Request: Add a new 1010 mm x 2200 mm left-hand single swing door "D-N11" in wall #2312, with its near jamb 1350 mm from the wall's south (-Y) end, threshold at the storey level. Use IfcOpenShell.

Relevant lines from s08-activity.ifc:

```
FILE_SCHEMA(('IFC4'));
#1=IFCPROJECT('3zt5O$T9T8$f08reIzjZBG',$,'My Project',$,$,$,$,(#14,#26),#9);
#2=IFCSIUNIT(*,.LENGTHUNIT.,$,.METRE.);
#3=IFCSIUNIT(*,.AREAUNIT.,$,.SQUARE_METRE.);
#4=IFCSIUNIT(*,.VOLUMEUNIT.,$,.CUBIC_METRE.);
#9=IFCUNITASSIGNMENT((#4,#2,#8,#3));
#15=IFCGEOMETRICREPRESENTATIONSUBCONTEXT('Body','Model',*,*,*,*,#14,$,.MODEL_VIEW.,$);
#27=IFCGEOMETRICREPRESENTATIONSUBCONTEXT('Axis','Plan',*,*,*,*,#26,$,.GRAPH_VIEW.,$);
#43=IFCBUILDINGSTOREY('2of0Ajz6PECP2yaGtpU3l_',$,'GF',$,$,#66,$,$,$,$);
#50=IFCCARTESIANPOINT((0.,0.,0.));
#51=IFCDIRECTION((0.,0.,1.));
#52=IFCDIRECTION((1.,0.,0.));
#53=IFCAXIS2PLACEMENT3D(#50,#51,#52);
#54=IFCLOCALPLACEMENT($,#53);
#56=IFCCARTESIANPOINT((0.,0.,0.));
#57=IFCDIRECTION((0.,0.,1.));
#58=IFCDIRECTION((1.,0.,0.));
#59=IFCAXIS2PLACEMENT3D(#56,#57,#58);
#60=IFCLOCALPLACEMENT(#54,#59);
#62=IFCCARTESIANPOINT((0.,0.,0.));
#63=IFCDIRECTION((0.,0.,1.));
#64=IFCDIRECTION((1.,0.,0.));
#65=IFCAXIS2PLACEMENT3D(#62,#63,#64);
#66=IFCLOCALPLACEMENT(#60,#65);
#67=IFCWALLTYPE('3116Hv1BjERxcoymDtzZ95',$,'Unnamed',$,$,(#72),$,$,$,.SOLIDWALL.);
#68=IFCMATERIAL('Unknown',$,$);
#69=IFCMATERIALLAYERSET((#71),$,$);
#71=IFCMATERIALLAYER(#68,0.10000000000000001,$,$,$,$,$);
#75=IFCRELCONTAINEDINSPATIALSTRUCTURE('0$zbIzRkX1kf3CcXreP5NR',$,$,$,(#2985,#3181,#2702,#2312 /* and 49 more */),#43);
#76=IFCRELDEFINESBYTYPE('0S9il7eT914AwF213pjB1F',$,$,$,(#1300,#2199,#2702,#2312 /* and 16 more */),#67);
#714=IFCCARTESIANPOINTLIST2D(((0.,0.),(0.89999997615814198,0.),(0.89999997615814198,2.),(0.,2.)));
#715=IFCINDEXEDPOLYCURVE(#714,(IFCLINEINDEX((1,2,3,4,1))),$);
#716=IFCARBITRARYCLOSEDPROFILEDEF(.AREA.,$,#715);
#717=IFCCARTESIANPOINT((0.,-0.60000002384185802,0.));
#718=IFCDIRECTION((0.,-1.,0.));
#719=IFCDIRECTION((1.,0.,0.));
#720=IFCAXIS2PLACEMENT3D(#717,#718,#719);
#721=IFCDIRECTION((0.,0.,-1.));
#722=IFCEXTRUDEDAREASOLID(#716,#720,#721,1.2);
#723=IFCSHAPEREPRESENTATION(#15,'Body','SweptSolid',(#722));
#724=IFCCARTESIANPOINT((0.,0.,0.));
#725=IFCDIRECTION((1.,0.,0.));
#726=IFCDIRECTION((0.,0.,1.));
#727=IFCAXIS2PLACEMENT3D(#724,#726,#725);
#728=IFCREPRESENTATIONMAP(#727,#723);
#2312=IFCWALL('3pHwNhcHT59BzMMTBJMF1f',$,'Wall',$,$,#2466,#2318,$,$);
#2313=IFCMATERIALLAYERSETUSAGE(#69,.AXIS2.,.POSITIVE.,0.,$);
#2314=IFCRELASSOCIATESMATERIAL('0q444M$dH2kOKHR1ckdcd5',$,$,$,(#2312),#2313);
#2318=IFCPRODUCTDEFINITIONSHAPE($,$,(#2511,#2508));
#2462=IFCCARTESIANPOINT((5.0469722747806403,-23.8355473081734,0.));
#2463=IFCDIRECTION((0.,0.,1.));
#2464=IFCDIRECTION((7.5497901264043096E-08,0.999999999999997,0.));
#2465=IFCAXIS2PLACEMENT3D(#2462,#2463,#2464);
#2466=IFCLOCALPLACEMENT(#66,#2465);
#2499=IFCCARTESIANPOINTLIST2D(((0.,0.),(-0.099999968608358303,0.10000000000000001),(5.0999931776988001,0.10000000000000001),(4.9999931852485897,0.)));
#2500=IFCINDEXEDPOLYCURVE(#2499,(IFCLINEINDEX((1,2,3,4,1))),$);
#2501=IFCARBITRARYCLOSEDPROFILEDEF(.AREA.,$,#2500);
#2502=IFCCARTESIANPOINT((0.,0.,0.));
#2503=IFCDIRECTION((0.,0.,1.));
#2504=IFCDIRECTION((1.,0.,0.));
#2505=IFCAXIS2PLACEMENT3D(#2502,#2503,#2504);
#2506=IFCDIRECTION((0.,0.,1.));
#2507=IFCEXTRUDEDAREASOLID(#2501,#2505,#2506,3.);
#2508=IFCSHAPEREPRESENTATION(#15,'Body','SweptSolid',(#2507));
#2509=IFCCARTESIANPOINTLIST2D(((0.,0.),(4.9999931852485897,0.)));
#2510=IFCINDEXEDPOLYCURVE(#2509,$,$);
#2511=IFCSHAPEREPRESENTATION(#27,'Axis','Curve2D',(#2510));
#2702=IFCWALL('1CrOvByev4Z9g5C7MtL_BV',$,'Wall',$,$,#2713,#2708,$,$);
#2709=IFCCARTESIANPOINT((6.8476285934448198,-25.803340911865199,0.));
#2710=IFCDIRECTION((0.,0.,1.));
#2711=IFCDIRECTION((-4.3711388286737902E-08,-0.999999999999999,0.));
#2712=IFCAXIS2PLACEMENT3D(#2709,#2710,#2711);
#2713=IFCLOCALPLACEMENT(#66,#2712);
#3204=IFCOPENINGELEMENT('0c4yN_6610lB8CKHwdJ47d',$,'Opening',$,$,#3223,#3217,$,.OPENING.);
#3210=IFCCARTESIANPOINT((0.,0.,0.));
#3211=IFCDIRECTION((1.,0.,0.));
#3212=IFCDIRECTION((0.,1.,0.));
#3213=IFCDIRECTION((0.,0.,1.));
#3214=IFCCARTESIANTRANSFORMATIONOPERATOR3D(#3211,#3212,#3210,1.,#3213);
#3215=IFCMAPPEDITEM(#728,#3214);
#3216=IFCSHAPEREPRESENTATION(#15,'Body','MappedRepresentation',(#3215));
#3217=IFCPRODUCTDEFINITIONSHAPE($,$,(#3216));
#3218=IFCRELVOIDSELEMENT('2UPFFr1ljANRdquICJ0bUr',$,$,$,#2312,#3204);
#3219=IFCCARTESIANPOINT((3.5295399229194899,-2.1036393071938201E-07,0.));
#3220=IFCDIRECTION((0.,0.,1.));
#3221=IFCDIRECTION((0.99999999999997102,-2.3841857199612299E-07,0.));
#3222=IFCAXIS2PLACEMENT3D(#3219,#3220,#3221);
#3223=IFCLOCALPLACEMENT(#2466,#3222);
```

```python
import numpy as np
import ifcopenshell
import ifcopenshell.api.feature
import ifcopenshell.api.geometry
import ifcopenshell.api.root
import ifcopenshell.api.spatial
import ifcopenshell.geom
import ifcopenshell.util.element
import ifcopenshell.util.placement
import ifcopenshell.util.representation
import ifcopenshell.util.shape
import ifcopenshell.util.unit

model = ifcopenshell.open("s08-activity.ifc")
unit_scale = ifcopenshell.util.unit.calculate_unit_scale(model)
settings = ifcopenshell.geom.settings()


def volume(element):
    """Net volume in cubic metres, openings subtracted."""
    shape = ifcopenshell.geom.create_shape(settings, element)
    return ifcopenshell.util.shape.get_volume(shape.geometry)


wall = model.by_guid("3pHwNhcHT59BzMMTBJMF1f")
storey = ifcopenshell.util.element.get_container(wall, ifc_class="IfcBuildingStorey")
context = ifcopenshell.util.representation.get_context(model, "Model", "Body", "MODEL_VIEW")
before = volume(wall)

width, height, from_end, sill = 1.01, 2.2, 1.35, 0.0  # metres

# The wall runs along its own X axis, and the end named is its -X end.
wall_shape = ifcopenshell.geom.create_shape(settings, wall)
x, y, z = ifcopenshell.util.shape.get_vertices(wall_shape.geometry).T
start = x.min() + from_end
face, thickness = float(y.min()), float(y.max() - y.min())
wall_matrix = ifcopenshell.util.placement.get_local_placement(wall.ObjectPlacement)
level = ifcopenshell.util.placement.get_local_placement(storey.ObjectPlacement)[2, 3]


def in_wall(x, y):
    """Placement at x, y metres in the wall's axes, at sill height."""
    matrix = wall_matrix.copy()
    matrix[:, 3] = wall_matrix @ np.array([x / unit_scale, y / unit_scale, 0.0, 1.0])
    matrix[2, 3] = level + sill / unit_scale
    return matrix


# Opening: a box that overshoots both wall faces by 50 mm.
opening = ifcopenshell.api.root.create_entity(model, ifc_class="IfcOpeningElement", predefined_type="OPENING")
box = ifcopenshell.api.geometry.add_wall_representation(
    model, context=context, length=width, height=height, thickness=thickness + 0.1
)
ifcopenshell.api.geometry.assign_representation(model, product=opening, representation=box)
ifcopenshell.api.geometry.edit_object_placement(model, product=opening, matrix=in_wall(start, face - 0.05), is_si=False)
ifcopenshell.api.feature.add_feature(model, feature=opening, element=wall)

door = ifcopenshell.api.root.create_entity(model, ifc_class="IfcDoor", name="D-N11", predefined_type="DOOR")
door.OverallWidth, door.OverallHeight = width / unit_scale, height / unit_scale
door.OperationType = "SINGLE_SWING_LEFT"
body = ifcopenshell.api.geometry.add_door_representation(
    model,
    context=context,
    overall_width=door.OverallWidth,
    overall_height=door.OverallHeight,
    operation_type="SINGLE_SWING_LEFT",
    lining_properties={"LiningDepth": thickness / unit_scale, "ThresholdDepth": thickness / unit_scale},
)
ifcopenshell.api.geometry.assign_representation(model, product=door, representation=body)
ifcopenshell.api.spatial.assign_container(model, products=[door], relating_structure=storey)
ifcopenshell.api.feature.add_filling(model, opening=opening, element=door)

# The lining spans the wall, so the door starts at the wall face.
ifcopenshell.api.geometry.edit_object_placement(model, product=door, matrix=in_wall(start, face), is_si=False)

after = volume(wall)

print(f"wall volume {before:.3f} -> {after:.3f} m3")

model.write("s08-activity_v2.ifc")
```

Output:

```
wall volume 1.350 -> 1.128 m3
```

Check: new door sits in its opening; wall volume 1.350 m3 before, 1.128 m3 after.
